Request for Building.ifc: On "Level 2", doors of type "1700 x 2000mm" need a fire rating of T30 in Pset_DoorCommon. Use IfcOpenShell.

First a look at what the model holds.

```python
import ifcopenshell
import ifcopenshell.util.element

model = ifcopenshell.open("Building.ifc")
print(model.schema)
storey = next(s for s in model.by_type("IfcBuildingStorey") if s.Name == "Level 2")
doors = [e for e in ifcopenshell.util.element.get_decomposition(storey) if e.is_a("IfcDoor")]
seen = {}
for e in doors:
    element_type = ifcopenshell.util.element.get_type(e)
    key = (element_type.Name if element_type != e and element_type else None, ifcopenshell.util.element.get_pset(e, "Pset_DoorCommon", "FireRating"))
    seen[key] = seen.get(key, 0) + 1
for (name, value), count in sorted(seen.items(), key=str):
    print(count, "x", name, "|", value)
```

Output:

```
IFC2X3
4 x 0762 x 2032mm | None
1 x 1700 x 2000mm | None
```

```python
import ifcopenshell
import ifcopenshell.api.pset
import ifcopenshell.util.element

model = ifcopenshell.open("Building.ifc")

storey = next(s for s in model.by_type("IfcBuildingStorey") if s.Name == "Level 2")
doors = [e for e in ifcopenshell.util.element.get_decomposition(storey) if e.is_a("IfcDoor")]

count = 0
for e in doors:
    element_type = ifcopenshell.util.element.get_type(e)
    if element_type in (None, e) or element_type.Name != "1700 x 2000mm":
        continue
    # add_pset returns the element's existing set when there is one.
    pset = ifcopenshell.api.pset.add_pset(model, product=e, name="Pset_DoorCommon")
    ifcopenshell.api.pset.edit_pset(model, pset=pset, properties={"FireRating": "T30"})
    count += 1

print(count, "doors updated")

model.write("Building-out.ifc")
```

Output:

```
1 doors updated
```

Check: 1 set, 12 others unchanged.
